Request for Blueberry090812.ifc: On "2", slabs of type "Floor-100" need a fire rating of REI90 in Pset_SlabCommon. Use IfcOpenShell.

First a look at what the model holds.

```python
import ifcopenshell
import ifcopenshell.util.element

model = ifcopenshell.open("Blueberry090812.ifc")
print(model.schema)
storey = next(s for s in model.by_type("IfcBuildingStorey") if s.Name == "2")
slabs = [e for e in ifcopenshell.util.element.get_decomposition(storey) if e.is_a("IfcSlab")]
seen = {}
for e in slabs:
    element_type = ifcopenshell.util.element.get_type(e)
    key = (element_type.Name if element_type != e and element_type else None, ifcopenshell.util.element.get_pset(e, "Pset_SlabCommon", "FireRating"))
    seen[key] = seen.get(key, 0) + 1
for (name, value), count in sorted(seen.items(), key=str):
    print(count, "x", name, "|", value)
```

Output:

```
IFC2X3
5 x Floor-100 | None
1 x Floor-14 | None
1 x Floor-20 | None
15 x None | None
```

```python
import ifcopenshell
import ifcopenshell.api.pset
import ifcopenshell.util.element

model = ifcopenshell.open("Blueberry090812.ifc")

storey = next(s for s in model.by_type("IfcBuildingStorey") if s.Name == "2")
slabs = [e for e in ifcopenshell.util.element.get_decomposition(storey) if e.is_a("IfcSlab")]

count = 0
for e in slabs:
    element_type = ifcopenshell.util.element.get_type(e)
    if element_type in (None, e) or element_type.Name != "Floor-100":
        continue
    found = ifcopenshell.util.element.get_pset(e, "Pset_SlabCommon", should_inherit=False)
    if found:
        pset = model.by_id(found["id"])
        if len(ifcopenshell.util.element.get_elements_by_pset(pset)) > 1:
            pset = ifcopenshell.api.pset.unshare_pset(model, products=[e], pset=pset)[0]
    else:
        pset = ifcopenshell.api.pset.add_pset(model, product=e, name="Pset_SlabCommon")
    ifcopenshell.api.pset.edit_pset(model, pset=pset, properties={"FireRating": "REI90"})
    count += 1

print(count, "slabs updated")

model.write("Blueberry090812-out.ifc")
```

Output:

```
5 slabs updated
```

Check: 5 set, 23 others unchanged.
